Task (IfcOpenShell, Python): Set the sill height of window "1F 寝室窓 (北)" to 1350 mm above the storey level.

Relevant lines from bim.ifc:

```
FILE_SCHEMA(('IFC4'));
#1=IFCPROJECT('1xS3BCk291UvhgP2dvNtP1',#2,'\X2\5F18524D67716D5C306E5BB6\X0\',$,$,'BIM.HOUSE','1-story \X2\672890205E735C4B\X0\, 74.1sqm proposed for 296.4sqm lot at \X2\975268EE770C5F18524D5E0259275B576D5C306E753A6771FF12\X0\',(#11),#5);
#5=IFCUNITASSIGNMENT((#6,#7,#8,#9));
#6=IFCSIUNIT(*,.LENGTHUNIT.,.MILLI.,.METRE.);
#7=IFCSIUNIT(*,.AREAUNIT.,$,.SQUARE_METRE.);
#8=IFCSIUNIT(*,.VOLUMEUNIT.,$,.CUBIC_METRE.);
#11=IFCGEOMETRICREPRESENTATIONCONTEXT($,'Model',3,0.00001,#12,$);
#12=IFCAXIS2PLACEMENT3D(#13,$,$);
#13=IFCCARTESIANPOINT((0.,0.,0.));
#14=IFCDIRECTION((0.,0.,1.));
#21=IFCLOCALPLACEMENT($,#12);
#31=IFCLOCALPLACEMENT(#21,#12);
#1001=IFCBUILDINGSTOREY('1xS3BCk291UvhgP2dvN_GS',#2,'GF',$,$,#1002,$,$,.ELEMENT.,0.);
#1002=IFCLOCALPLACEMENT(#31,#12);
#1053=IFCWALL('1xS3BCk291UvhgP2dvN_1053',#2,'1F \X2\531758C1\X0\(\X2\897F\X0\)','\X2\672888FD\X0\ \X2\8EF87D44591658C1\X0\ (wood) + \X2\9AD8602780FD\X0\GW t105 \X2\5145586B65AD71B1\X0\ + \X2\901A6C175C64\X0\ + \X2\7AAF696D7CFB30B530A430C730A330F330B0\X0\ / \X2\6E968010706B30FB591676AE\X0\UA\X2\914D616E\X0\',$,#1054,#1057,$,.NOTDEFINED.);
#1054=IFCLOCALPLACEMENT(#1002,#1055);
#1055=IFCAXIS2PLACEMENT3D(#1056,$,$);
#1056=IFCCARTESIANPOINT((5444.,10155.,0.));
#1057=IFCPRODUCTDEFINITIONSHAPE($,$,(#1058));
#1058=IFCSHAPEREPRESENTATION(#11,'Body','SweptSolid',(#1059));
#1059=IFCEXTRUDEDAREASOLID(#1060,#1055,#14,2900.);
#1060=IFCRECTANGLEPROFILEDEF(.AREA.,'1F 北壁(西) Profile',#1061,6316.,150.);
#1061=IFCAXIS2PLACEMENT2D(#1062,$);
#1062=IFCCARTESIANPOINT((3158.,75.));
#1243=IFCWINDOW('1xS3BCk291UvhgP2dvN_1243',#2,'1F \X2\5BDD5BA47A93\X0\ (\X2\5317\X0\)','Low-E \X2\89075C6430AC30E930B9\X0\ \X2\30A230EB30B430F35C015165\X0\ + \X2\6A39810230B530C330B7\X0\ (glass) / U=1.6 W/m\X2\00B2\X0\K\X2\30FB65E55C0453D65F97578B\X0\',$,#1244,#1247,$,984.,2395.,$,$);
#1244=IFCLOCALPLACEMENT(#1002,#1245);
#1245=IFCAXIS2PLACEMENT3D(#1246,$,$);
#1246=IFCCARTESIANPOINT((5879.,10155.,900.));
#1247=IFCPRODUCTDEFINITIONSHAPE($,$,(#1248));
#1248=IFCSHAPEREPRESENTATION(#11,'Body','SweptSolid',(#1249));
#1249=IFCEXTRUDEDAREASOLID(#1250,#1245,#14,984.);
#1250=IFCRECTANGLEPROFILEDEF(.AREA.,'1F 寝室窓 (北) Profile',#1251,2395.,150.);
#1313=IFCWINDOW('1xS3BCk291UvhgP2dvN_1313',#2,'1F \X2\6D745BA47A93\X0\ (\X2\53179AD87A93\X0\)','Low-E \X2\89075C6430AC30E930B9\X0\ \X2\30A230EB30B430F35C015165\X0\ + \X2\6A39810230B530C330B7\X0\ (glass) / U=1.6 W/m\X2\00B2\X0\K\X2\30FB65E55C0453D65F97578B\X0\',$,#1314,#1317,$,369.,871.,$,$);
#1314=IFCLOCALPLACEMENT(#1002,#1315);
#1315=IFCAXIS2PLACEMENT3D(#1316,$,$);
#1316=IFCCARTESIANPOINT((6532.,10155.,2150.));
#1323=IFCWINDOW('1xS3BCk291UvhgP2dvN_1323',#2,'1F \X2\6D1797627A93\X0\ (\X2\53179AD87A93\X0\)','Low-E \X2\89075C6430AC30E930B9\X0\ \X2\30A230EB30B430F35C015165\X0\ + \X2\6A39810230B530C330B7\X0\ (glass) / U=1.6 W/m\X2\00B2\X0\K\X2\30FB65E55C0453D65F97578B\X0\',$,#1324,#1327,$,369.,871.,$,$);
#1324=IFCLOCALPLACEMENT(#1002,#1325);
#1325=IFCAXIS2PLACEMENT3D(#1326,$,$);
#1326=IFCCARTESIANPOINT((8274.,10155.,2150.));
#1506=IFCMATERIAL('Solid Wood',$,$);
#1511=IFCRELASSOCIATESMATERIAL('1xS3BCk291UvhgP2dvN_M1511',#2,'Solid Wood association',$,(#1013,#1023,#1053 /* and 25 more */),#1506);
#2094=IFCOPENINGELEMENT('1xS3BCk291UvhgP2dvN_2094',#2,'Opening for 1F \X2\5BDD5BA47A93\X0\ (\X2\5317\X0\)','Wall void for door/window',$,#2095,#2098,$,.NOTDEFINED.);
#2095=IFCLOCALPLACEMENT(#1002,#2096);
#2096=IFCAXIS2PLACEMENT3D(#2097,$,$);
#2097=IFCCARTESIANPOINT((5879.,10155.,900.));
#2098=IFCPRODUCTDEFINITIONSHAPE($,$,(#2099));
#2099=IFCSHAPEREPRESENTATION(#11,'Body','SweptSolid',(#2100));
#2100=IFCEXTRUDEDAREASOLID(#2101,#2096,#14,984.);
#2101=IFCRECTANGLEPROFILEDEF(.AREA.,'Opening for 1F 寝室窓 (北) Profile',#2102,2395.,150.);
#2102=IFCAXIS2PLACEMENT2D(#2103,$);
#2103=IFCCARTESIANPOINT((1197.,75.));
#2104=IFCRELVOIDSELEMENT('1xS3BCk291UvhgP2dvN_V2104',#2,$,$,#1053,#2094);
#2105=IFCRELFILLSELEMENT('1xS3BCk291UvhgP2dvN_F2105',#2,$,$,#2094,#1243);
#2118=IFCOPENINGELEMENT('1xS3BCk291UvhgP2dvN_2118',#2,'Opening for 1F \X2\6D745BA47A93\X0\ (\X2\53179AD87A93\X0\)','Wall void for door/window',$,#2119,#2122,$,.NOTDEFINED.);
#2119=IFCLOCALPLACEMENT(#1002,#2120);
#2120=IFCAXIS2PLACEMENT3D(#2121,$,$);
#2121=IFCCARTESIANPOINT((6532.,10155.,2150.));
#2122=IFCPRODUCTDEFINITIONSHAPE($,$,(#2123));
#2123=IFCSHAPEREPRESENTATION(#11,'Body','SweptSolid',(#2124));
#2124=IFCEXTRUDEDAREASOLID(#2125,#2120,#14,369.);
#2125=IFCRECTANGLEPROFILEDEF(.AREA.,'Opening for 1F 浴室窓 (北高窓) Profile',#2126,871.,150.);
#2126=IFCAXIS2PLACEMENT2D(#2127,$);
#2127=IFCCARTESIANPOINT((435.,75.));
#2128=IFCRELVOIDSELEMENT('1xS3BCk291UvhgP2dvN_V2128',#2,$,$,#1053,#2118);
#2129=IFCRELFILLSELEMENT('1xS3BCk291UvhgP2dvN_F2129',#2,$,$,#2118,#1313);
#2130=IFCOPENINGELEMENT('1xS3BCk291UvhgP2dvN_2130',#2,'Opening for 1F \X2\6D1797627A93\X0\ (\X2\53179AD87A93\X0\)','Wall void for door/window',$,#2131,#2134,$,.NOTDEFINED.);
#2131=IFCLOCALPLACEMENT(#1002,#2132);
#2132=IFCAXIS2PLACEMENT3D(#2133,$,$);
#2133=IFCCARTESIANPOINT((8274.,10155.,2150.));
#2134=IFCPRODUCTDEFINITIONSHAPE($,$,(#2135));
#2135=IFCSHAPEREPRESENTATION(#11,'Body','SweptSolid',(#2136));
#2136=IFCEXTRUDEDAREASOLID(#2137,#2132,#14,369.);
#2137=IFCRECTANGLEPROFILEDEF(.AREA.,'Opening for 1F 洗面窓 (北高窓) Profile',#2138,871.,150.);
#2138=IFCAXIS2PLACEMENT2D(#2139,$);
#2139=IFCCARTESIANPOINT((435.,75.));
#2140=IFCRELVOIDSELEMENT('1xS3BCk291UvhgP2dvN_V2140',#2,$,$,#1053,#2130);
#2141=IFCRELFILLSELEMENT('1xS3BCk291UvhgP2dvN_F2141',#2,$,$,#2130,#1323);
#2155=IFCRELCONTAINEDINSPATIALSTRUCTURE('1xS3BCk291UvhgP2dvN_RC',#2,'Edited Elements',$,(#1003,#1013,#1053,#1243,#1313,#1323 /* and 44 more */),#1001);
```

```python
import numpy as np
import ifcopenshell
import ifcopenshell.api.geometry
import ifcopenshell.geom
import ifcopenshell.util.element
import ifcopenshell.util.placement
import ifcopenshell.util.shape
import ifcopenshell.util.unit

model = ifcopenshell.open("bim.ifc")
unit_scale = ifcopenshell.util.unit.calculate_unit_scale(model)

window = model.by_id(1243)
opening = window.FillsVoids[0].RelatingOpeningElement
storey = ifcopenshell.util.element.get_container(window, ifc_class="IfcBuildingStorey")
level = ifcopenshell.util.placement.get_local_placement(storey.ObjectPlacement)[2, 3]

# The opening's origin need not be at the sill, so measure its lowest point.
shape = ifcopenshell.geom.create_shape(ifcopenshell.geom.settings(), opening)
bottom = ifcopenshell.util.shape.get_shape_bottom_elevation(shape, shape.geometry) / unit_scale
dz = level + 1350.0 - bottom

shift = np.array([0.0, 0.0, dz])
# The window is not placed relative to its opening, so move both.
for product in (opening, window):
    matrix = ifcopenshell.util.placement.get_local_placement(product.ObjectPlacement)
    matrix[:3, 3] += shift
    ifcopenshell.api.geometry.edit_object_placement(model, product=product, matrix=matrix, is_si=False)

print(f"moved by {dz * unit_scale:+.3f} m")

model.write("bim_v2.ifc")
```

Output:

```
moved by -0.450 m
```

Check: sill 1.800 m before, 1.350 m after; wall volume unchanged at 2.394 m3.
